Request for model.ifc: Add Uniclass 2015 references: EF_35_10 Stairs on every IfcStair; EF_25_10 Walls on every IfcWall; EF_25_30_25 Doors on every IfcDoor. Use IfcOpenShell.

First a look at what the model holds.

```python
import ifcopenshell

model = ifcopenshell.open("model.ifc")
print(model.schema)
print("classifications:", [c.Name for c in model.by_type("IfcClassification")])
for ifc_class in ("IfcDoor", "IfcRoof", "IfcStair", "IfcWall", "IfcWindow"):
    print(ifc_class, len(model.by_type(ifc_class)))
```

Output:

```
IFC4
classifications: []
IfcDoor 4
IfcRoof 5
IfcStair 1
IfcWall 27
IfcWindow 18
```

```python
import ifcopenshell
import ifcopenshell.api.classification

model = ifcopenshell.open("model.ifc")

system = ifcopenshell.api.classification.add_classification(model, classification="Uniclass 2015")

codes = {
    "IfcStair": ("EF_35_10", "Stairs"),
    "IfcWall": ("EF_25_10", "Walls"),
    "IfcDoor": ("EF_25_30_25", "Doors"),
}
for ifc_class, (code, name) in codes.items():
    products = model.by_type(ifc_class)
    ifcopenshell.api.classification.add_reference(
        model, products=products, classification=system, identification=code, name=name
    )
    print(code, len(products))

model.write("model-out.ifc")
```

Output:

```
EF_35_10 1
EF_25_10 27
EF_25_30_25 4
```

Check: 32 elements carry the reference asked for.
